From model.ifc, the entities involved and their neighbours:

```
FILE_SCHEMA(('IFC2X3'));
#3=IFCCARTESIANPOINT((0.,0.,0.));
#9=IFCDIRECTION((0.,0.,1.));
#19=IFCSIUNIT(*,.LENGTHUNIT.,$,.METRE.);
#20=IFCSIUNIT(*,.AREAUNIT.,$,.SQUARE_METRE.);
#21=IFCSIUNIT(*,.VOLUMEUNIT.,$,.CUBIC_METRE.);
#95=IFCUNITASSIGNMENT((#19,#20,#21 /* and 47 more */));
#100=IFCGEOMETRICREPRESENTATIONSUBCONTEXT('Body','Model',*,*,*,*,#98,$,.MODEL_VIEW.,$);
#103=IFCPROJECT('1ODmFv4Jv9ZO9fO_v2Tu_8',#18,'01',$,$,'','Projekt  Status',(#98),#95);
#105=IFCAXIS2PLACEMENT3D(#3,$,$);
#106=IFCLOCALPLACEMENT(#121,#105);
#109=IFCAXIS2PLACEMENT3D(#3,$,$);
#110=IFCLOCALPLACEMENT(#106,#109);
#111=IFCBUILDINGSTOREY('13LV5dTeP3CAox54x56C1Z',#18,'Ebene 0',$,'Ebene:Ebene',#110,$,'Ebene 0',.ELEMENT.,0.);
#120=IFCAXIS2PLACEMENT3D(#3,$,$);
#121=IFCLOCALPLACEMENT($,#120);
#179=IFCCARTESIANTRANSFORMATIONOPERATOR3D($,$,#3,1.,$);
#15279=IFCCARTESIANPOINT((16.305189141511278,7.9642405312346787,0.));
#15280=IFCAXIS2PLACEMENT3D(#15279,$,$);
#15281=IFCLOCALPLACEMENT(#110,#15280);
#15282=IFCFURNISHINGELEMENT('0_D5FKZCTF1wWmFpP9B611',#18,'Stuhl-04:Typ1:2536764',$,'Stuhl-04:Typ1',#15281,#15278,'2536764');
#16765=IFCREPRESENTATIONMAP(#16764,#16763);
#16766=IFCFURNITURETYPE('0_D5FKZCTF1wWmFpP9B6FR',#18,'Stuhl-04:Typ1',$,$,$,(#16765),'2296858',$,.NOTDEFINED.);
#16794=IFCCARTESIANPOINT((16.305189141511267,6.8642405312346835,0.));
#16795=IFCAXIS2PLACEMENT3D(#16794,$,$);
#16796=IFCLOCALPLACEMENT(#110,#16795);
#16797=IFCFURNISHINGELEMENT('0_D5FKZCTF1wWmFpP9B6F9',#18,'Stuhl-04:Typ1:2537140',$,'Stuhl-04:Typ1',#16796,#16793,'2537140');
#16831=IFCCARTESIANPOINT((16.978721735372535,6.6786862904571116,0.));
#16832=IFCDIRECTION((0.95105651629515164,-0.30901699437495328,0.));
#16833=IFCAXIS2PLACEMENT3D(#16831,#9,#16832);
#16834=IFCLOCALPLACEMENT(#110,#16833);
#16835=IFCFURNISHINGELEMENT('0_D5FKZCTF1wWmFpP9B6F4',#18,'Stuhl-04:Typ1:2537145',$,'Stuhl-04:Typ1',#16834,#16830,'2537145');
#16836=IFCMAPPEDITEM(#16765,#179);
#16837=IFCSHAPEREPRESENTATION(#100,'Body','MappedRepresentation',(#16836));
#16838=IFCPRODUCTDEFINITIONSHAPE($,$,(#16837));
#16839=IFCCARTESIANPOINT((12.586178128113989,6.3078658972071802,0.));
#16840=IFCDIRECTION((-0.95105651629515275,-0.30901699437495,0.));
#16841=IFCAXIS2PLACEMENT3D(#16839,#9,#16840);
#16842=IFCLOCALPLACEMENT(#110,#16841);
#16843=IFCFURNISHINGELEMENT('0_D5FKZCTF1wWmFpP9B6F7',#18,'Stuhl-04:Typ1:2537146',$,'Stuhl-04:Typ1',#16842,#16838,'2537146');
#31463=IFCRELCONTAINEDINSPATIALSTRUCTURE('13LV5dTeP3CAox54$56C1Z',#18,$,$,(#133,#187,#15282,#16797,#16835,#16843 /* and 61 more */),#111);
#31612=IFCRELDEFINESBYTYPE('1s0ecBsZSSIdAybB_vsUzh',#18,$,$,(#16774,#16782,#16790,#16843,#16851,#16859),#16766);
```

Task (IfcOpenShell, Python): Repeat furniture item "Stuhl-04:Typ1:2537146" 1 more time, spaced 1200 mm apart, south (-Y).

```python
import numpy as np
import ifcopenshell
import ifcopenshell.api.geometry
import ifcopenshell.api.root
import ifcopenshell.util.element
import ifcopenshell.util.placement

model = ifcopenshell.open("model.ifc")

source = model.by_guid("0_D5FKZCTF1wWmFpP9B6F7")
base = ifcopenshell.util.placement.get_local_placement(source.ObjectPlacement)
step = np.array([0.0, -1.0, 0.0]) * 1.2

for i in range(1, 2):
    copy = ifcopenshell.api.root.copy_class(model, product=source)
    copy.Representation = ifcopenshell.util.element.copy_deep(
        model, source.Representation, exclude=["IfcGeometricRepresentationContext", "IfcRepresentationMap"]
    )
    copy.Name = "Stuhl-04:Typ1"
    copy.Tag = None
    matrix = base.copy()
    matrix[:3, 3] += i * step
    print("added at", matrix[:3, 3].round(3) + 0.0)
    ifcopenshell.api.geometry.edit_object_placement(model, product=copy, matrix=matrix, is_si=False)

model.write("model_edited.ifc")
```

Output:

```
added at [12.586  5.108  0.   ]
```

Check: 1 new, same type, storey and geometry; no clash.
